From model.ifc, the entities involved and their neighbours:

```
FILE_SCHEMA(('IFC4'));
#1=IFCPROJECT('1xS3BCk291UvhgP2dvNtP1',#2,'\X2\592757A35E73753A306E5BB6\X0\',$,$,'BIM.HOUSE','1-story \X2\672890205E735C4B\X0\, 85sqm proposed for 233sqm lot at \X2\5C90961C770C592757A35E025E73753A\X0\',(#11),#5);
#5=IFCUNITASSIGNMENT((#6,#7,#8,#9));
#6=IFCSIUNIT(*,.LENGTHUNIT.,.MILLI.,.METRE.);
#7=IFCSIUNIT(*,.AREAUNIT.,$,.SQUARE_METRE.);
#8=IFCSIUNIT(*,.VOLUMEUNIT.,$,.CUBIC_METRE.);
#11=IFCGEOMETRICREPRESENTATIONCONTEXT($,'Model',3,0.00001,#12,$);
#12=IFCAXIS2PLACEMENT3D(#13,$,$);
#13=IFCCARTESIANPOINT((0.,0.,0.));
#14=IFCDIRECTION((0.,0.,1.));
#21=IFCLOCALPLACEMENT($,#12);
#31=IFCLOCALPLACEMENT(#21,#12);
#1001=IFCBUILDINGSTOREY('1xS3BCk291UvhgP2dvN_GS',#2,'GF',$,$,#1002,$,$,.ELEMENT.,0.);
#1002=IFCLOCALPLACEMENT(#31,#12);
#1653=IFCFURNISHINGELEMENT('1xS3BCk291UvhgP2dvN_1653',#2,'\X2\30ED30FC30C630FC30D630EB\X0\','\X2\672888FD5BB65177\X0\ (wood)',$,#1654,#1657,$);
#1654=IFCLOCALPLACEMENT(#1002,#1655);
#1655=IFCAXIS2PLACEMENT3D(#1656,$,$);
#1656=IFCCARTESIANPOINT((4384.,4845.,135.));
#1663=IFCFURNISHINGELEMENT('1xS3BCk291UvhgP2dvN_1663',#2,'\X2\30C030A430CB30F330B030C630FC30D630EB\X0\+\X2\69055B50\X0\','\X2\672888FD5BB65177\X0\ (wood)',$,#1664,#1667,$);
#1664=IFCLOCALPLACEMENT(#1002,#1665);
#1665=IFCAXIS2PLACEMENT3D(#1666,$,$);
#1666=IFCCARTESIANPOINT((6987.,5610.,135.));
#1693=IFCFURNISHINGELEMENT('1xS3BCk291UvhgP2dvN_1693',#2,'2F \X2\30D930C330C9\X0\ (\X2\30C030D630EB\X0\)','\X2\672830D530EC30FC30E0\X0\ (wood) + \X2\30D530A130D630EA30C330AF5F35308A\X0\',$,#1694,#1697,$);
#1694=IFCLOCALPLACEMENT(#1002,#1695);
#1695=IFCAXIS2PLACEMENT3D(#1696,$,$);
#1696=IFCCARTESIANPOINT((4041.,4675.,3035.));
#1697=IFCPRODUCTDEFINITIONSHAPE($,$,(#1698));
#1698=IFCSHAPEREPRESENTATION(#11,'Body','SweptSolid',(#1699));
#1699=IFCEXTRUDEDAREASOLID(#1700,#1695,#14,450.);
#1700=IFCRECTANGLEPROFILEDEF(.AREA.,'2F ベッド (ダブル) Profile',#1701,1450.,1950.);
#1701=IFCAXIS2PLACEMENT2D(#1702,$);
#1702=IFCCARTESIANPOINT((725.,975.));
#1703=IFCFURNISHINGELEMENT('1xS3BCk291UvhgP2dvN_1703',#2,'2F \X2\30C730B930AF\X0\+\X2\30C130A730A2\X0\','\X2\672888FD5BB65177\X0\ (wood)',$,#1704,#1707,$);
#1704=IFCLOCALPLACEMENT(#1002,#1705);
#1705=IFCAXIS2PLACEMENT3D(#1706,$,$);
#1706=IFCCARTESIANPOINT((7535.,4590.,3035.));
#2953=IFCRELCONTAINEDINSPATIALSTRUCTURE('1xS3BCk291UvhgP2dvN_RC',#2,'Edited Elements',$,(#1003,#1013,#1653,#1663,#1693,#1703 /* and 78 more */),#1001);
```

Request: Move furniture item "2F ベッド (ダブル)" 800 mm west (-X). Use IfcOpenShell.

```python
import ifcopenshell
import ifcopenshell.api.geometry
import ifcopenshell.util.placement

model = ifcopenshell.open("model.ifc")

item = model.by_guid("1xS3BCk291UvhgP2dvN_1693")
matrix = ifcopenshell.util.placement.get_local_placement(item.ObjectPlacement)
matrix[0, 3] -= 800.0
ifcopenshell.api.geometry.edit_object_placement(model, product=item, matrix=matrix, is_si=False)

print(ifcopenshell.util.placement.get_local_placement(item.ObjectPlacement).round(3) + 0.0)

model.write("model_edited.ifc")
```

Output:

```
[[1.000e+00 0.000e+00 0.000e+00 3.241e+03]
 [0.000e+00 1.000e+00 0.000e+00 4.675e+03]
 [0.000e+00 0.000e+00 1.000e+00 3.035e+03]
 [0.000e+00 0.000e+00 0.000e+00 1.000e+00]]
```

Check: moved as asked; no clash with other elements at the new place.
